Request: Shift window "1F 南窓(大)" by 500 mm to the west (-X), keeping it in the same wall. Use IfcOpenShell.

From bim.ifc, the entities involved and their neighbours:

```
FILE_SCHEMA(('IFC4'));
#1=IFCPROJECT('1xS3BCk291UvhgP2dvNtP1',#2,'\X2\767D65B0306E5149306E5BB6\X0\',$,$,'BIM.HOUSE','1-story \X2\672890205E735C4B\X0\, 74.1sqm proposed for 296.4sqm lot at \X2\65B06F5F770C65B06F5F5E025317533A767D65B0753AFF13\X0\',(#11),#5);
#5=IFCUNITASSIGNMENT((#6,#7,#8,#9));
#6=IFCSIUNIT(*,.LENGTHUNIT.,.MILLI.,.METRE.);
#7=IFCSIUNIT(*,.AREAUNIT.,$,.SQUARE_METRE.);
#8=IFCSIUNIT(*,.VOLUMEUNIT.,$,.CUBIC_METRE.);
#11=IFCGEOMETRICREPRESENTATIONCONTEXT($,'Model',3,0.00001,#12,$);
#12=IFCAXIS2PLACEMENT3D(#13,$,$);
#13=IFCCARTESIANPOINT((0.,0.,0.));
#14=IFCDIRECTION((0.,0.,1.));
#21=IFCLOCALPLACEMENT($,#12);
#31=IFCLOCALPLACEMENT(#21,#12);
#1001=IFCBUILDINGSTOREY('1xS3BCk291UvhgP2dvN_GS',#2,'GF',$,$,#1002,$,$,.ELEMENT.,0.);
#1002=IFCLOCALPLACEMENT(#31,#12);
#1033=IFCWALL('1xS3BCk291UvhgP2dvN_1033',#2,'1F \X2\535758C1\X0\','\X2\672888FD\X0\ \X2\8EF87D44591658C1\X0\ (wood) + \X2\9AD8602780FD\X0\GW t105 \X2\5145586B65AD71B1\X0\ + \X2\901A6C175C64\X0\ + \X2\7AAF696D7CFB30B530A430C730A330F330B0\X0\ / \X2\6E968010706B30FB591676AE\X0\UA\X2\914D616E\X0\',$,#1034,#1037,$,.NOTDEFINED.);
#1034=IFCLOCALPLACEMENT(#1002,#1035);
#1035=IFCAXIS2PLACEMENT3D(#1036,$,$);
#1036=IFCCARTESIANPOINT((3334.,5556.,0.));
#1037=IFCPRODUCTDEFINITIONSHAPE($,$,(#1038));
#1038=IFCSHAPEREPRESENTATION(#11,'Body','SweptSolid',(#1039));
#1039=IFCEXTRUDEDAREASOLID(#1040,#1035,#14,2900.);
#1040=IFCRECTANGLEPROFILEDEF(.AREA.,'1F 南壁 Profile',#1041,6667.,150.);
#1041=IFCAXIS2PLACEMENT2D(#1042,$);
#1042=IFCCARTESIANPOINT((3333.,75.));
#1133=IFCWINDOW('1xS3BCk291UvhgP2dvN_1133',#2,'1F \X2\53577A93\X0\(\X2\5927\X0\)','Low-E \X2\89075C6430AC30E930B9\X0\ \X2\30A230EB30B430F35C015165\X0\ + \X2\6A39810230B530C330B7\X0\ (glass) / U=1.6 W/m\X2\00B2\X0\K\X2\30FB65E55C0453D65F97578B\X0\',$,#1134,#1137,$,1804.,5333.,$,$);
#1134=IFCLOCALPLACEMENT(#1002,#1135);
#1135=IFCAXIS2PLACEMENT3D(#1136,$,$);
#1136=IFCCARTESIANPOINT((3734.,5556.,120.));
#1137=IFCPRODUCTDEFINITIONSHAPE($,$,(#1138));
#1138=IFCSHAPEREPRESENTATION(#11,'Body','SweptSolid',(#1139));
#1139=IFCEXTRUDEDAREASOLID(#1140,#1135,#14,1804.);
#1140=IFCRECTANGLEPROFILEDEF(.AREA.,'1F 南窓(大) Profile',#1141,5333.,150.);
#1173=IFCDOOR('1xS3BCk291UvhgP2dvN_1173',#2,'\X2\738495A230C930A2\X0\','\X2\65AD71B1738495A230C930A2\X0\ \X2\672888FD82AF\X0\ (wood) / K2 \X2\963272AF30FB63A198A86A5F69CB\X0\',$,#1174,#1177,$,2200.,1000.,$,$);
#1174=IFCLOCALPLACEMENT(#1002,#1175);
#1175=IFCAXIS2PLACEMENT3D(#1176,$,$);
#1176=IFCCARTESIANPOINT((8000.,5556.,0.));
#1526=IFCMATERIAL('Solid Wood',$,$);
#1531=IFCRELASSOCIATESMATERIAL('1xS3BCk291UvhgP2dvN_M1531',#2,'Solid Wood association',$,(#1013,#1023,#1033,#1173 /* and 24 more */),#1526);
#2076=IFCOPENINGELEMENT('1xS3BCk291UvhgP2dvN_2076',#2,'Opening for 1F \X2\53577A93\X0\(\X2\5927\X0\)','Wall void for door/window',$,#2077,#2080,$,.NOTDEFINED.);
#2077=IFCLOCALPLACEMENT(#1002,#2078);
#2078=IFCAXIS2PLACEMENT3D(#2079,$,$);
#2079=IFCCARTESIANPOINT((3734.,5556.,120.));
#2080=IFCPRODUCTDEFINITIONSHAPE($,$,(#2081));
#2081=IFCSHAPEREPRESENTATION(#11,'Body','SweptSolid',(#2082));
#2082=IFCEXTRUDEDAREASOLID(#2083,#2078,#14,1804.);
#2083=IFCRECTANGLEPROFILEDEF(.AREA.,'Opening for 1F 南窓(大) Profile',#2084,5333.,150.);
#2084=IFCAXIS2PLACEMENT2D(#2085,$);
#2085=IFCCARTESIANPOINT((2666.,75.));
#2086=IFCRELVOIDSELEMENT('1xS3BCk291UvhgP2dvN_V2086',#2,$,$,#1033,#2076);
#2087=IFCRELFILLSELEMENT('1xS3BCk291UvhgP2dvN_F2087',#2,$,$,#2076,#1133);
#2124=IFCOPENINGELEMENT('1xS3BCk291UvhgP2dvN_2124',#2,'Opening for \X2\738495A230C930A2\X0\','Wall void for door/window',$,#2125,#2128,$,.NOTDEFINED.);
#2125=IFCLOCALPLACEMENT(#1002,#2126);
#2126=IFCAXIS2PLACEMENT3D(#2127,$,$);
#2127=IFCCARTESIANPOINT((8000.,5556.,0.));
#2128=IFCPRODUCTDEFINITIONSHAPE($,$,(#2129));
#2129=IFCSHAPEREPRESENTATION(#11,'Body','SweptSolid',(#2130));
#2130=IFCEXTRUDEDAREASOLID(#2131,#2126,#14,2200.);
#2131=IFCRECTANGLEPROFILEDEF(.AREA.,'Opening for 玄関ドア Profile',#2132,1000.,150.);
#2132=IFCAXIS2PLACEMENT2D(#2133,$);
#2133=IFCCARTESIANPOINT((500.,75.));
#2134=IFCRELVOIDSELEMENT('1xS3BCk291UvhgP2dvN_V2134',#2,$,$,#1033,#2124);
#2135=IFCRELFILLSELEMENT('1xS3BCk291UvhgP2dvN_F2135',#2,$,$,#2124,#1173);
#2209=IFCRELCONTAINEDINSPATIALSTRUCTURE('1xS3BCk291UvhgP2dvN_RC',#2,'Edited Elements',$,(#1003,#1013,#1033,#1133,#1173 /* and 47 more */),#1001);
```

```python
import ifcopenshell
import ifcopenshell.api.geometry
import ifcopenshell.util.placement
import ifcopenshell.util.unit

model = ifcopenshell.open("bim.ifc")
unit_scale = ifcopenshell.util.unit.calculate_unit_scale(model)

window = model.by_guid("1xS3BCk291UvhgP2dvN_1133")
opening = window.FillsVoids[0].RelatingOpeningElement
wall = opening.VoidsElements[0].RelatingBuildingElement

wall_matrix = ifcopenshell.util.placement.get_local_placement(wall.ObjectPlacement)
shift = wall_matrix[:3, 0] * -0.5 / unit_scale
before = ifcopenshell.util.placement.get_local_placement(window.ObjectPlacement)[:3, 3].copy()

# The window is not placed relative to its opening, so move both.
for product in (opening, window):
    matrix = ifcopenshell.util.placement.get_local_placement(product.ObjectPlacement)
    matrix[:3, 3] += shift
    ifcopenshell.api.geometry.edit_object_placement(model, product=product, matrix=matrix, is_si=False)

after = ifcopenshell.util.placement.get_local_placement(window.ObjectPlacement)[:3, 3]
print("window moved by", (after - before).round(3) + 0.0)

model.write("bim_rev.ifc")
```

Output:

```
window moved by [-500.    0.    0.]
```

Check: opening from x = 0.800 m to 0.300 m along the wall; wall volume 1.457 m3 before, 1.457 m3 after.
